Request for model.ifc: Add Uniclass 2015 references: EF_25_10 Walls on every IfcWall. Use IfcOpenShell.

First a look at what the model holds.

```python
import ifcopenshell

model = ifcopenshell.open("model.ifc")
print(model.schema)
print("classifications:", [c.Name for c in model.by_type("IfcClassification")])
for ifc_class in ("IfcDoor", "IfcRoof", "IfcStair", "IfcWall", "IfcWindow"):
    print(ifc_class, len(model.by_type(ifc_class)))
```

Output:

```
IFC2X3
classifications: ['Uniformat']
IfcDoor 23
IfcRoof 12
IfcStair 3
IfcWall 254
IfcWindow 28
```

```python
import ifcopenshell
import ifcopenshell.api.classification

model = ifcopenshell.open("model.ifc")

# IFC2X3 requires Source and Edition and has no link from the project to the system.
system = model.create_entity("IfcClassification", Source="NBS", Edition="2015", Name="Uniclass 2015")

codes = {
    "IfcWall": ("EF_25_10", "Walls"),
}
for ifc_class, (code, name) in codes.items():
    products = model.by_type(ifc_class)
    ifcopenshell.api.classification.add_reference(
        model, products=products, classification=system, identification=code, name=name
    )
    print(code, len(products))

model.write("model_edited.ifc")
```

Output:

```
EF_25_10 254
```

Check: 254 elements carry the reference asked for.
